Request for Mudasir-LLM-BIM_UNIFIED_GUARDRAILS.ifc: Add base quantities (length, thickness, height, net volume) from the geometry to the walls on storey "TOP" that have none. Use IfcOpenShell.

First a look at what the model holds.

```python
import ifcopenshell
import ifcopenshell.util.element
import ifcopenshell.util.unit

model = ifcopenshell.open("Mudasir-LLM-BIM_UNIFIED_GUARDRAILS.ifc")
print(model.schema)
for unit_type in ("LENGTHUNIT", "AREAUNIT", "VOLUMEUNIT"):
    print(unit_type, ifcopenshell.util.unit.calculate_unit_scale(model, unit_type))
storey = next(s for s in model.by_type("IfcBuildingStorey") if s.Name == "TOP")
walls = [e for e in ifcopenshell.util.element.get_decomposition(storey) if e.is_a("IfcWall")]
for e in sorted(walls, key=lambda e: e.id()):
    print(e.id(), e.is_a(), e.Name, list(ifcopenshell.util.element.get_psets(e, qtos_only=True)), sep=" | ")
```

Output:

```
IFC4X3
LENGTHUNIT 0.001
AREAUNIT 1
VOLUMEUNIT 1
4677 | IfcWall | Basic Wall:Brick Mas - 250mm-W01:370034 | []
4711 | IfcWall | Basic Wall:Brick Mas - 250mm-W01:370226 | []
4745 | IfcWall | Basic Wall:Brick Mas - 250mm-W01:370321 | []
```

```python
import ifcopenshell
import ifcopenshell.api.pset
import ifcopenshell.geom
import ifcopenshell.util.element
import ifcopenshell.util.shape
import ifcopenshell.util.unit

model = ifcopenshell.open("Mudasir-LLM-BIM_UNIFIED_GUARDRAILS.ifc")
unit_scale = ifcopenshell.util.unit.calculate_unit_scale(model)
volume_scale = ifcopenshell.util.unit.calculate_unit_scale(model, "VOLUMEUNIT")
settings = ifcopenshell.geom.settings()

storey = next(s for s in model.by_type("IfcBuildingStorey") if s.Name == "TOP")
walls = [e for e in ifcopenshell.util.element.get_decomposition(storey) if e.is_a("IfcWall")]

for e in sorted(walls, key=lambda e: e.id()):
    if ifcopenshell.util.element.get_psets(e, qtos_only=True, should_inherit=False):
        continue
    # Geometry comes back in metres, in the element's own axes.
    shape = ifcopenshell.geom.create_shape(settings, e)
    values = {
        "Length": ifcopenshell.util.shape.get_x(shape.geometry) / unit_scale,
        "Width": ifcopenshell.util.shape.get_y(shape.geometry) / unit_scale,
        "Height": ifcopenshell.util.shape.get_z(shape.geometry) / unit_scale,
        "NetVolume": ifcopenshell.util.shape.get_volume(shape.geometry) / volume_scale,
    }
    qto = ifcopenshell.api.pset.add_qto(model, product=e, name="Qto_WallBaseQuantities")
    ifcopenshell.api.pset.edit_qto(model, qto=qto, properties=values)
    print(e.id(), {k: round(v, 3) for k, v in values.items()})

model.write("Mudasir-LLM-BIM_UNIFIED_GUARDRAILS_rev.ifc")
```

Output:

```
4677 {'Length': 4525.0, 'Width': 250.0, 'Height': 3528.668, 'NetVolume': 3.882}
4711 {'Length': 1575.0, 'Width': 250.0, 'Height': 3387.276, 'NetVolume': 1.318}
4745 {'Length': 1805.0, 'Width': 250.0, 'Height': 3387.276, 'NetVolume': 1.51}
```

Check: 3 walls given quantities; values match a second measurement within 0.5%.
